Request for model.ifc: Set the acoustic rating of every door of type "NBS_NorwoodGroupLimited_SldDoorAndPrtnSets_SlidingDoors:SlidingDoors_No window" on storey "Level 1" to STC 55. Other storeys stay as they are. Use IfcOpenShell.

First a look at what the model holds.

```python
import ifcopenshell
import ifcopenshell.util.element

model = ifcopenshell.open("model.ifc")
print(model.schema)
storey = next(s for s in model.by_type("IfcBuildingStorey") if s.Name == "Level 1")
doors = [e for e in ifcopenshell.util.element.get_decomposition(storey) if e.is_a("IfcDoor")]
seen = {}
for e in doors:
    element_type = ifcopenshell.util.element.get_type(e)
    key = (element_type.Name if element_type != e and element_type else None, ifcopenshell.util.element.get_pset(e, "Pset_DoorCommon", "AcousticRating"))
    seen[key] = seen.get(key, 0) + 1
for (name, value), count in sorted(seen.items(), key=str):
    print(count, "x", name, "|", value)
```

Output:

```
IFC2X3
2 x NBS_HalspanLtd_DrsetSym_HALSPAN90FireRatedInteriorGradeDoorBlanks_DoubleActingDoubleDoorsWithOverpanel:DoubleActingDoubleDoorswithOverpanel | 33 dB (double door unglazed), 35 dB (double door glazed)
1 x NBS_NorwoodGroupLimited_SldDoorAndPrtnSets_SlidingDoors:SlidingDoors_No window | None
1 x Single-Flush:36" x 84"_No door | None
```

```python
import ifcopenshell
import ifcopenshell.api.pset
import ifcopenshell.util.element

model = ifcopenshell.open("model.ifc")

storey = next(s for s in model.by_type("IfcBuildingStorey") if s.Name == "Level 1")
doors = [e for e in ifcopenshell.util.element.get_decomposition(storey) if e.is_a("IfcDoor")]

count = 0
for e in doors:
    element_type = ifcopenshell.util.element.get_type(e)
    if element_type in (None, e) or element_type.Name != "NBS_NorwoodGroupLimited_SldDoorAndPrtnSets_SlidingDoors:SlidingDoors_No window":
        continue
    # add_pset returns the element's existing set when there is one.
    pset = ifcopenshell.api.pset.add_pset(model, product=e, name="Pset_DoorCommon")
    ifcopenshell.api.pset.edit_pset(model, pset=pset, properties={"AcousticRating": "STC 55"})
    count += 1

print(count, "doors updated")

model.write("model_rev.ifc")
```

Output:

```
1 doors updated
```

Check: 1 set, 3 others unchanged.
